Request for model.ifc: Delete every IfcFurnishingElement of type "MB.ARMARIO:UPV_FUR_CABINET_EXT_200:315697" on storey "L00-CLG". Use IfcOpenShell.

First a look at what the model holds.

```python
import ifcopenshell
import ifcopenshell.util.element

model = ifcopenshell.open("model.ifc")
print(model.schema)
storey = next(s for s in model.by_type("IfcBuildingStorey") if s.Name == "L00-CLG")
furniture = [e for e in ifcopenshell.util.element.get_decomposition(storey) if e.is_a("IfcFurnishingElement")]
seen = {}
for e in furniture:
    element_type = ifcopenshell.util.element.get_type(e)
    name = element_type.Name if element_type not in (None, e) else None
    seen[name] = seen.get(name, 0) + 1
for name, count in sorted(seen.items(), key=str):
    print(count, "x", name)
```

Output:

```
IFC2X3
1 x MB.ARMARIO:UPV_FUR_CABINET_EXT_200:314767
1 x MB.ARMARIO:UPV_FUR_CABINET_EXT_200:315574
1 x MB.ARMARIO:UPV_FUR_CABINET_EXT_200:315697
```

```python
import ifcopenshell
import ifcopenshell.api.root
import ifcopenshell.util.element

model = ifcopenshell.open("model.ifc")

storey = next(s for s in model.by_type("IfcBuildingStorey") if s.Name == "L00-CLG")
furniture = [e for e in ifcopenshell.util.element.get_decomposition(storey) if e.is_a("IfcFurnishingElement")]
targets = [e for e in furniture if (t := ifcopenshell.util.element.get_type(e)) not in (None, e) and t.Name == "MB.ARMARIO:UPV_FUR_CABINET_EXT_200:315697"]

for e in targets:
    ifcopenshell.api.root.remove_product(model, product=e)
print(len(targets), "removed")

model.write("model_v2.ifc")
```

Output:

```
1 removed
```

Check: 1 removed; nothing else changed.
